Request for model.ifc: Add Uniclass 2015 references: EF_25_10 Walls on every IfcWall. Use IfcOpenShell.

First a look at what the model holds.

```python
import ifcopenshell

model = ifcopenshell.open("model.ifc")
print(model.schema)
print("classifications:", [c.Name for c in model.by_type("IfcClassification")])
for ifc_class in ("IfcDoor", "IfcRoof", "IfcStair", "IfcWall", "IfcWindow"):
    print(ifc_class, len(model.by_type(ifc_class)))
```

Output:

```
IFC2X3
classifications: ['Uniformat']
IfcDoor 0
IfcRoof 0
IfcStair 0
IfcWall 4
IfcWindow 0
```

```python
import ifcopenshell
import ifcopenshell.api.classification

model = ifcopenshell.open("model.ifc")

# IFC2X3 requires Source and Edition and has no link from the project to the system.
system = model.create_entity("IfcClassification", Source="NBS", Edition="2015", Name="Uniclass 2015")

codes = {
    "IfcWall": ("EF_25_10", "Walls"),
}
for ifc_class, (code, name) in codes.items():
    products = model.by_type(ifc_class)
    ifcopenshell.api.classification.add_reference(
        model, products=products, classification=system, identification=code, name=name
    )
    print(code, len(products))

model.write("model_v2.ifc")
```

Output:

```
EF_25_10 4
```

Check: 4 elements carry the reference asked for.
